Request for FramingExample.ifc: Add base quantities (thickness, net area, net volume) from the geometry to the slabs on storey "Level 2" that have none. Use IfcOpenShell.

First a look at what the model holds.

```python
import ifcopenshell
import ifcopenshell.util.element
import ifcopenshell.util.unit

model = ifcopenshell.open("FramingExample.ifc")
print(model.schema)
for unit_type in ("LENGTHUNIT", "AREAUNIT", "VOLUMEUNIT"):
    print(unit_type, ifcopenshell.util.unit.calculate_unit_scale(model, unit_type))
storey = next(s for s in model.by_type("IfcBuildingStorey") if s.Name == "Level 2")
slabs = [e for e in ifcopenshell.util.element.get_decomposition(storey) if e.is_a("IfcSlab")]
for e in sorted(slabs, key=lambda e: e.id()):
    print(e.id(), e.is_a(), e.Name, list(ifcopenshell.util.element.get_psets(e, qtos_only=True)), sep=" | ")
```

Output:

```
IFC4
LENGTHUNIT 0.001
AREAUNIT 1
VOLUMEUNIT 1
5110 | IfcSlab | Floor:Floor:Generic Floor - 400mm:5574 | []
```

```python
import ifcopenshell
import ifcopenshell.api.pset
import ifcopenshell.geom
import ifcopenshell.util.element
import ifcopenshell.util.shape
import ifcopenshell.util.unit

model = ifcopenshell.open("FramingExample.ifc")
unit_scale = ifcopenshell.util.unit.calculate_unit_scale(model)
area_scale = ifcopenshell.util.unit.calculate_unit_scale(model, "AREAUNIT")
volume_scale = ifcopenshell.util.unit.calculate_unit_scale(model, "VOLUMEUNIT")
settings = ifcopenshell.geom.settings()

storey = next(s for s in model.by_type("IfcBuildingStorey") if s.Name == "Level 2")
slabs = [e for e in ifcopenshell.util.element.get_decomposition(storey) if e.is_a("IfcSlab")]

for e in sorted(slabs, key=lambda e: e.id()):
    if ifcopenshell.util.element.get_psets(e, qtos_only=True, should_inherit=False):
        continue
    # Geometry comes back in metres, in the element's own axes.
    shape = ifcopenshell.geom.create_shape(settings, e)
    values = {
        "Width": ifcopenshell.util.shape.get_z(shape.geometry) / unit_scale,
        "NetArea": ifcopenshell.util.shape.get_footprint_area(shape.geometry) / area_scale,
        "NetVolume": ifcopenshell.util.shape.get_volume(shape.geometry) / volume_scale,
    }
    qto = ifcopenshell.api.pset.add_qto(model, product=e, name="Qto_SlabBaseQuantities")
    ifcopenshell.api.pset.edit_qto(model, qto=qto, properties=values)
    print(e.id(), {k: round(v, 3) for k, v in values.items()})

model.write("FramingExample_rev.ifc")
```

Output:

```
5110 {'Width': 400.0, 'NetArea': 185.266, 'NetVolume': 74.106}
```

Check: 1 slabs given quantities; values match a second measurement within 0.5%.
